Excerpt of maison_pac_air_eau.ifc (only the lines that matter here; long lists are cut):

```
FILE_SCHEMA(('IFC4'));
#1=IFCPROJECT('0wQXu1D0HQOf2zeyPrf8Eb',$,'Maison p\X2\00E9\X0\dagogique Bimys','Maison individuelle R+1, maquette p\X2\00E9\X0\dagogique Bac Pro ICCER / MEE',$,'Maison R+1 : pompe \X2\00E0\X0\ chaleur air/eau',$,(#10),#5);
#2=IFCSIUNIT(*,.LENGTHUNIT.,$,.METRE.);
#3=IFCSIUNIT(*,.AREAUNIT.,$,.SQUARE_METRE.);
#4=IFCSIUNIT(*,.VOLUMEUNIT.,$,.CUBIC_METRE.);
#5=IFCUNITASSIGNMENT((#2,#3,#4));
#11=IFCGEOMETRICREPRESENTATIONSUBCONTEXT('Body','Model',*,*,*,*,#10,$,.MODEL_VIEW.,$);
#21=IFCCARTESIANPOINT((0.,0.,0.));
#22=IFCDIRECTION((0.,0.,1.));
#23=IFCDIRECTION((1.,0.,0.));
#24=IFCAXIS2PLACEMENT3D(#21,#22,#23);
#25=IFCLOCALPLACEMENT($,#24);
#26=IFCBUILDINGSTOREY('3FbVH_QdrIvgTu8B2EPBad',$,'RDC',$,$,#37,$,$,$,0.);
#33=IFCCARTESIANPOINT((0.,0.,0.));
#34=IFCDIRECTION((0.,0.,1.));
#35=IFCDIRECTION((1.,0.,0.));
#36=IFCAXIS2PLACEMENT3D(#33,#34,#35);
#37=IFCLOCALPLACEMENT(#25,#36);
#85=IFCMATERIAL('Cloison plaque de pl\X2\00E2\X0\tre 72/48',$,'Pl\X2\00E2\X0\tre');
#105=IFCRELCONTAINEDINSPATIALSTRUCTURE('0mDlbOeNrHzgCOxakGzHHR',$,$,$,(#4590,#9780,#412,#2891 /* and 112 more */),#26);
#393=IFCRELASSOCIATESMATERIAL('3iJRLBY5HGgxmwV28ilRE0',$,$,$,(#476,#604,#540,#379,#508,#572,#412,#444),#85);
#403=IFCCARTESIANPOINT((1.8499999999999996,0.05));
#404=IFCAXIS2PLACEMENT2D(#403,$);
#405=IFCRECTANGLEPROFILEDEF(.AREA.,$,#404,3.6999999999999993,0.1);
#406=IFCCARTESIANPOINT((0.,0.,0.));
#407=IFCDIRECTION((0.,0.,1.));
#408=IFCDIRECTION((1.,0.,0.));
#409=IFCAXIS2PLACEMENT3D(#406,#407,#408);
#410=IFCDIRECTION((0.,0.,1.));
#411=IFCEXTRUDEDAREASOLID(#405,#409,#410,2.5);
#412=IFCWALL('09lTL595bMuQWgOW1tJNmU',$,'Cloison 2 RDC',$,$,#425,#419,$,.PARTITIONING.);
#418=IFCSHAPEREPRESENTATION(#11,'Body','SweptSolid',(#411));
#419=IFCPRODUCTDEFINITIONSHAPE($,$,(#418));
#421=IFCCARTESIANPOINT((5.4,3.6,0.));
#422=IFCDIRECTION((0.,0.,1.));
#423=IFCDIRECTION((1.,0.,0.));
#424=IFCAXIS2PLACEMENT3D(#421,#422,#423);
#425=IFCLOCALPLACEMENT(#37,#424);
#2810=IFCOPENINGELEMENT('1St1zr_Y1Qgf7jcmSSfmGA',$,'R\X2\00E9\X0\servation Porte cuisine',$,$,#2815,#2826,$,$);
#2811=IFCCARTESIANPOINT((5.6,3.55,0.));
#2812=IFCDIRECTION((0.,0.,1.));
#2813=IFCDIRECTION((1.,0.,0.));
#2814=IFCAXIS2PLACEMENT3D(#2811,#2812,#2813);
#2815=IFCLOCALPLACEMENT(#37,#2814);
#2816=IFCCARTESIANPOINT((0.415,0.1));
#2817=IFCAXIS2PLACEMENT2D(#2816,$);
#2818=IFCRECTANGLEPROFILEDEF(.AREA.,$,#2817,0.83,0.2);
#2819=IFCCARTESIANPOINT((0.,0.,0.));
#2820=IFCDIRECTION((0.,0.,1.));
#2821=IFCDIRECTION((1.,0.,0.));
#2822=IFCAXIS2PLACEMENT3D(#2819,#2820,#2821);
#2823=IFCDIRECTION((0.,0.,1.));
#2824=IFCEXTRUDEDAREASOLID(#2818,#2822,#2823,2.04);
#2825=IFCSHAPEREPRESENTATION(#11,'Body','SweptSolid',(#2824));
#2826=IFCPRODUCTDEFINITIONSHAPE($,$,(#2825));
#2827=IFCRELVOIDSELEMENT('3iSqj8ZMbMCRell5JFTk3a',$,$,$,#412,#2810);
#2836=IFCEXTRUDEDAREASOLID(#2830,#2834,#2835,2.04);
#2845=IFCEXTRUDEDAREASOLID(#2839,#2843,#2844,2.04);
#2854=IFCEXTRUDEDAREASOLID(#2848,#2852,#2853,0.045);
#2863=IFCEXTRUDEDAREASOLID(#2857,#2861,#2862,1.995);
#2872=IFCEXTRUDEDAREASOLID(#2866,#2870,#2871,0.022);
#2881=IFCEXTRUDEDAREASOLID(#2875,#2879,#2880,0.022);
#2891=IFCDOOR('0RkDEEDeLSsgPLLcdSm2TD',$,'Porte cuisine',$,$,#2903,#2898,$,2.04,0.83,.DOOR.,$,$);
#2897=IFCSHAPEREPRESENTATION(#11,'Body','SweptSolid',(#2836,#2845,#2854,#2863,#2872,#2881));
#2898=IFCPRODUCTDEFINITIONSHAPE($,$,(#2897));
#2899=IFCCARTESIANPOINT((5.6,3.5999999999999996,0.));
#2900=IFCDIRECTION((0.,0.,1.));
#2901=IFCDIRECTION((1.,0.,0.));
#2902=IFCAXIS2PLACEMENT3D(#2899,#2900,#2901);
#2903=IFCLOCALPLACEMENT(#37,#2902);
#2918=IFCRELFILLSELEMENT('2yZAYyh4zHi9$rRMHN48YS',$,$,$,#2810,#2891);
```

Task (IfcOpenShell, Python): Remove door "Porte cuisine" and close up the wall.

```python
import ifcopenshell
import ifcopenshell.api.feature
import ifcopenshell.api.root
import ifcopenshell.geom
import ifcopenshell.util.shape

model = ifcopenshell.open("maison_pac_air_eau.ifc")
settings = ifcopenshell.geom.settings()


def volume(element):
    """Net volume in cubic metres, openings subtracted."""
    shape = ifcopenshell.geom.create_shape(settings, element)
    return ifcopenshell.util.shape.get_volume(shape.geometry)


door = model.by_guid("0RkDEEDeLSsgPLLcdSm2TD")
opening = door.FillsVoids[0].RelatingOpeningElement
wall = opening.VoidsElements[0].RelatingBuildingElement
before = volume(wall)

ifcopenshell.api.root.remove_product(model, product=door)
ifcopenshell.api.feature.remove_feature(model, feature=opening)

after = volume(wall)

print(f"wall volume {before:.3f} -> {after:.3f} m3")

model.write("maison_pac_air_eau_v2.ifc")
```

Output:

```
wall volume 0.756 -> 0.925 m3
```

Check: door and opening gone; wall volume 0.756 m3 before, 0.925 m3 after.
